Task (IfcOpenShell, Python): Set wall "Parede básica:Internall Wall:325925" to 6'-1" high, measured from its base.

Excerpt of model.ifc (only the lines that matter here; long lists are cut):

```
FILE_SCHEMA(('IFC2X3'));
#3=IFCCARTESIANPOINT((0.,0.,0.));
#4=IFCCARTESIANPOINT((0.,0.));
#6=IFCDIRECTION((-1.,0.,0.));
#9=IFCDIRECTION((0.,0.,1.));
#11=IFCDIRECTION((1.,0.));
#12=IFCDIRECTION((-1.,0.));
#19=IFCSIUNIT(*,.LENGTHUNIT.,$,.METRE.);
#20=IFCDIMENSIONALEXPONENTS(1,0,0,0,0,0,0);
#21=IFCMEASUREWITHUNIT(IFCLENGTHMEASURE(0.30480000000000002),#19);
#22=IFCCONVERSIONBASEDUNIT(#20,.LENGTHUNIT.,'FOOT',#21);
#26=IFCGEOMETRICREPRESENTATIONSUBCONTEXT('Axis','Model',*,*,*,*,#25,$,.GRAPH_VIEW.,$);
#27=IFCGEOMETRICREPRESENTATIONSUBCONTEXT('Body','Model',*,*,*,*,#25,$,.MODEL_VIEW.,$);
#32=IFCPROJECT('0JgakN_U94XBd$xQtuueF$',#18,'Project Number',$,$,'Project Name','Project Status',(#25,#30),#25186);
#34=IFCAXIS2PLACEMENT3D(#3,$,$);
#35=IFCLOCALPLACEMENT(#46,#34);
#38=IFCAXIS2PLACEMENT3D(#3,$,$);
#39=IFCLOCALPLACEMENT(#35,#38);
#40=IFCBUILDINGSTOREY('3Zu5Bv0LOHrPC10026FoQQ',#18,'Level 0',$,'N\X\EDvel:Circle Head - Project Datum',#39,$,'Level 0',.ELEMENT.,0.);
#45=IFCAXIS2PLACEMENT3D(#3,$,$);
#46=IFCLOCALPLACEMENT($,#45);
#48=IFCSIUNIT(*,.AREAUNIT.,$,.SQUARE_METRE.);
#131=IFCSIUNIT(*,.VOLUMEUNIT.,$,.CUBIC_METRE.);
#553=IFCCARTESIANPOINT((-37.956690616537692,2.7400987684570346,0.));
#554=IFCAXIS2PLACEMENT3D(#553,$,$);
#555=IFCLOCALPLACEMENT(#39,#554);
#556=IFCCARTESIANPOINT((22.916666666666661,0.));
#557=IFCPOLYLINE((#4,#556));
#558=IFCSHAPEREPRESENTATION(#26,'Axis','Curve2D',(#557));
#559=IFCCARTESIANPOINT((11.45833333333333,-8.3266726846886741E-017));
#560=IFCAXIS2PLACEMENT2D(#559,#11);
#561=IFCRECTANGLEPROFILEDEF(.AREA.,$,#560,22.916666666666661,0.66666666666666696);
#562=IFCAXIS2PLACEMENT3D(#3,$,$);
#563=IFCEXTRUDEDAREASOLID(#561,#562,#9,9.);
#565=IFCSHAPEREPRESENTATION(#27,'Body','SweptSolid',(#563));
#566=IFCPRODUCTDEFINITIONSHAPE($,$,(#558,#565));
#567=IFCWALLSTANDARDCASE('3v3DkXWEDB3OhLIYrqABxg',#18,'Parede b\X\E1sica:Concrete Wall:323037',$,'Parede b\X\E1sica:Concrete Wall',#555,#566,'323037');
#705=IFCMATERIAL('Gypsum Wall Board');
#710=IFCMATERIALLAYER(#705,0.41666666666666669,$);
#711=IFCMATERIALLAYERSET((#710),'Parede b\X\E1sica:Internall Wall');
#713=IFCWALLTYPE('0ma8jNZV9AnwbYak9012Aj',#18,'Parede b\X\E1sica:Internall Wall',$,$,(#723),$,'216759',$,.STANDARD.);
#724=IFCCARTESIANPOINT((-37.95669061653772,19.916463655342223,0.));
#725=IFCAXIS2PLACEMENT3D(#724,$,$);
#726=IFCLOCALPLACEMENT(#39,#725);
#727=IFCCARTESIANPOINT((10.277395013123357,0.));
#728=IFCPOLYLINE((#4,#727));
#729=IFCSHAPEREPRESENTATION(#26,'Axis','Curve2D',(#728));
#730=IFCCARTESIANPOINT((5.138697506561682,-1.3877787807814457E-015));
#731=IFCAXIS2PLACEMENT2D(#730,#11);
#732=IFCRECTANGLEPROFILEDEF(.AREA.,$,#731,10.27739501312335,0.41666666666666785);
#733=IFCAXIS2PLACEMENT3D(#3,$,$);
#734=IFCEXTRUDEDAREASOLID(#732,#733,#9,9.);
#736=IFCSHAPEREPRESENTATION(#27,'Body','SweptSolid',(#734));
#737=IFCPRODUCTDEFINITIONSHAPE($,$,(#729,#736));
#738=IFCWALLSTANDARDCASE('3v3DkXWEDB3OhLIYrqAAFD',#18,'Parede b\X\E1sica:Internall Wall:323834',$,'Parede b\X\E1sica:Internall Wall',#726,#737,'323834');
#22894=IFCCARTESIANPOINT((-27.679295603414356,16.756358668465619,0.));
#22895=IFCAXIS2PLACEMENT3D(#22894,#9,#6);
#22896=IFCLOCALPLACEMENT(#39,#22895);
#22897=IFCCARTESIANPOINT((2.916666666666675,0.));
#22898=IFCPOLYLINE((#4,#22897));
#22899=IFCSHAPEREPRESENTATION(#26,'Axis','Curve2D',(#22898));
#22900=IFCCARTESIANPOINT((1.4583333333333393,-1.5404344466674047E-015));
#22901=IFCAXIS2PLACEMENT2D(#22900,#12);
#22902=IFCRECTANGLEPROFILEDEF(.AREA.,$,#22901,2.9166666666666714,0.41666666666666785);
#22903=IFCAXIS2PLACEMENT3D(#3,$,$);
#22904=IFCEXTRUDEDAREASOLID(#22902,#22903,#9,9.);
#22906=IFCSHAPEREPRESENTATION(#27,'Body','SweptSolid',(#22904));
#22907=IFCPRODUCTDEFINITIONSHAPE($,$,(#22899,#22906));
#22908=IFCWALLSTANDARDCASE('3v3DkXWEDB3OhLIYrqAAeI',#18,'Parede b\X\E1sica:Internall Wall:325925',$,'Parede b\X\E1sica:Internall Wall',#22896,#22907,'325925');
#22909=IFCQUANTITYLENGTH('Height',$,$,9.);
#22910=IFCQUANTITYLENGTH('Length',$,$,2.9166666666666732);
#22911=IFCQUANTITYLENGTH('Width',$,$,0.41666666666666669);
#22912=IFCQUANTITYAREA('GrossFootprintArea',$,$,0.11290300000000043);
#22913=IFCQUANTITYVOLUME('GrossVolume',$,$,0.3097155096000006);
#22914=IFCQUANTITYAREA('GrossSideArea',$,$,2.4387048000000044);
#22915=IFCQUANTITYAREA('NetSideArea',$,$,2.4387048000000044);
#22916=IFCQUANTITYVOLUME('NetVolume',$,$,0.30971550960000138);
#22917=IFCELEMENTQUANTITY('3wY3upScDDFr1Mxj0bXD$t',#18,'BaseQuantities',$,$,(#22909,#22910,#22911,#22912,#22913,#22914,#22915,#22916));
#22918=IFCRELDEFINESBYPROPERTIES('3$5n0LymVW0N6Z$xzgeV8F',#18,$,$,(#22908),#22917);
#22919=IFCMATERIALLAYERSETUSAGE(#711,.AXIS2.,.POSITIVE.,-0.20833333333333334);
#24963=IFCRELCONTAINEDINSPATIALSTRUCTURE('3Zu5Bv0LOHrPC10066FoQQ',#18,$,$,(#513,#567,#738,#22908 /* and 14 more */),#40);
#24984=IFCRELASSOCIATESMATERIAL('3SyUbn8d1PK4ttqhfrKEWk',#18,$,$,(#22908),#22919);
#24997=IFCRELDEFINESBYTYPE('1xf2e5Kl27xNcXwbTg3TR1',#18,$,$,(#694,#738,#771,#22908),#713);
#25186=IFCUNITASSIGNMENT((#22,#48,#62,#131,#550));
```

```python
import ifcopenshell
import ifcopenshell.api.pset
import ifcopenshell.geom
import ifcopenshell.util.element
import ifcopenshell.util.representation
import ifcopenshell.util.shape
import ifcopenshell.util.unit

model = ifcopenshell.open("model.ifc")
unit_scale = ifcopenshell.util.unit.calculate_unit_scale(model)
area_scale = ifcopenshell.util.unit.calculate_unit_scale(model, "AREAUNIT")
volume_scale = ifcopenshell.util.unit.calculate_unit_scale(model, "VOLUMEUNIT")
settings = ifcopenshell.geom.settings()


def volume(element):
    """Net volume in cubic metres, openings subtracted."""
    shape = ifcopenshell.geom.create_shape(settings, element)
    return ifcopenshell.util.shape.get_volume(shape.geometry)


wall = model.by_guid("3v3DkXWEDB3OhLIYrqAAeI")
before = volume(wall)

body = ifcopenshell.util.representation.get_representation(wall, "Model", "Body")
solid = body.Items[0]
old_height = solid.Depth
solid.Depth = 73 * 0.0254 / unit_scale
after = volume(wall)
thickness = 0.127  # wall thickness in metres

# Update the stored height, areas and volumes.
qto = model.by_id(ifcopenshell.util.element.get_pset(wall, "BaseQuantities", should_inherit=False)["id"])
ifcopenshell.api.pset.edit_qto(model, qto=qto, properties={
    "Height": solid.Depth,
    "GrossVolume": ifcopenshell.util.element.get_pset(wall, "BaseQuantities", "GrossVolume") * solid.Depth / old_height,
    "GrossSideArea": ifcopenshell.util.element.get_pset(wall, "BaseQuantities", "GrossSideArea") * solid.Depth / old_height,
    "NetSideArea": after / thickness / area_scale,
    "NetVolume": after / volume_scale,
})

print(f"height {old_height:g} -> {solid.Depth:g}, volume {before:.3f} -> {after:.3f} m3")

model.write("model_rev.ifc")
```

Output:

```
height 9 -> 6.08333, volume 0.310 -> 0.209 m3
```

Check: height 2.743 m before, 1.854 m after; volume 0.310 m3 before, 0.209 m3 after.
